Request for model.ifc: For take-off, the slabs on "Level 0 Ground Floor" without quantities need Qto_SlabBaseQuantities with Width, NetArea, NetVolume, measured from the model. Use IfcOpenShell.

First a look at what the model holds.

```python
import ifcopenshell
import ifcopenshell.util.element
import ifcopenshell.util.unit

model = ifcopenshell.open("model.ifc")
print(model.schema)
for unit_type in ("LENGTHUNIT", "AREAUNIT", "VOLUMEUNIT"):
    print(unit_type, ifcopenshell.util.unit.calculate_unit_scale(model, unit_type))
storey = next(s for s in model.by_type("IfcBuildingStorey") if s.Name == "Level 0 Ground Floor")
slabs = [e for e in ifcopenshell.util.element.get_decomposition(storey) if e.is_a("IfcSlab")]
for e in sorted(slabs, key=lambda e: e.id()):
    print(e.id(), e.is_a(), e.Name, list(ifcopenshell.util.element.get_psets(e, qtos_only=True)), sep=" | ")
```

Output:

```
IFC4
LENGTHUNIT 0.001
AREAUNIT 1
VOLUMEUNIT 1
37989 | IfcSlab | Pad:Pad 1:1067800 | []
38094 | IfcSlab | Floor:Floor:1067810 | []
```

```python
import ifcopenshell
import ifcopenshell.api.pset
import ifcopenshell.geom
import ifcopenshell.util.element
import ifcopenshell.util.shape
import ifcopenshell.util.unit

model = ifcopenshell.open("model.ifc")
unit_scale = ifcopenshell.util.unit.calculate_unit_scale(model)
area_scale = ifcopenshell.util.unit.calculate_unit_scale(model, "AREAUNIT")
volume_scale = ifcopenshell.util.unit.calculate_unit_scale(model, "VOLUMEUNIT")
settings = ifcopenshell.geom.settings()

storey = next(s for s in model.by_type("IfcBuildingStorey") if s.Name == "Level 0 Ground Floor")
slabs = [e for e in ifcopenshell.util.element.get_decomposition(storey) if e.is_a("IfcSlab")]

for e in sorted(slabs, key=lambda e: e.id()):
    if ifcopenshell.util.element.get_psets(e, qtos_only=True, should_inherit=False):
        continue
    # Geometry comes back in metres, in the element's own axes.
    shape = ifcopenshell.geom.create_shape(settings, e)
    values = {
        "Width": ifcopenshell.util.shape.get_z(shape.geometry) / unit_scale,
        "NetArea": ifcopenshell.util.shape.get_footprint_area(shape.geometry) / area_scale,
        "NetVolume": ifcopenshell.util.shape.get_volume(shape.geometry) / volume_scale,
    }
    qto = ifcopenshell.api.pset.add_qto(model, product=e, name="Qto_SlabBaseQuantities")
    ifcopenshell.api.pset.edit_qto(model, qto=qto, properties=values)
    print(e.id(), {k: round(v, 3) for k, v in values.items()})

model.write("model_rev.ifc")
```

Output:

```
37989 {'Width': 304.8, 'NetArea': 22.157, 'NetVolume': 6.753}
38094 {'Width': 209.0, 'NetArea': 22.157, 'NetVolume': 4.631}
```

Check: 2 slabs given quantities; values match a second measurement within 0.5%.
